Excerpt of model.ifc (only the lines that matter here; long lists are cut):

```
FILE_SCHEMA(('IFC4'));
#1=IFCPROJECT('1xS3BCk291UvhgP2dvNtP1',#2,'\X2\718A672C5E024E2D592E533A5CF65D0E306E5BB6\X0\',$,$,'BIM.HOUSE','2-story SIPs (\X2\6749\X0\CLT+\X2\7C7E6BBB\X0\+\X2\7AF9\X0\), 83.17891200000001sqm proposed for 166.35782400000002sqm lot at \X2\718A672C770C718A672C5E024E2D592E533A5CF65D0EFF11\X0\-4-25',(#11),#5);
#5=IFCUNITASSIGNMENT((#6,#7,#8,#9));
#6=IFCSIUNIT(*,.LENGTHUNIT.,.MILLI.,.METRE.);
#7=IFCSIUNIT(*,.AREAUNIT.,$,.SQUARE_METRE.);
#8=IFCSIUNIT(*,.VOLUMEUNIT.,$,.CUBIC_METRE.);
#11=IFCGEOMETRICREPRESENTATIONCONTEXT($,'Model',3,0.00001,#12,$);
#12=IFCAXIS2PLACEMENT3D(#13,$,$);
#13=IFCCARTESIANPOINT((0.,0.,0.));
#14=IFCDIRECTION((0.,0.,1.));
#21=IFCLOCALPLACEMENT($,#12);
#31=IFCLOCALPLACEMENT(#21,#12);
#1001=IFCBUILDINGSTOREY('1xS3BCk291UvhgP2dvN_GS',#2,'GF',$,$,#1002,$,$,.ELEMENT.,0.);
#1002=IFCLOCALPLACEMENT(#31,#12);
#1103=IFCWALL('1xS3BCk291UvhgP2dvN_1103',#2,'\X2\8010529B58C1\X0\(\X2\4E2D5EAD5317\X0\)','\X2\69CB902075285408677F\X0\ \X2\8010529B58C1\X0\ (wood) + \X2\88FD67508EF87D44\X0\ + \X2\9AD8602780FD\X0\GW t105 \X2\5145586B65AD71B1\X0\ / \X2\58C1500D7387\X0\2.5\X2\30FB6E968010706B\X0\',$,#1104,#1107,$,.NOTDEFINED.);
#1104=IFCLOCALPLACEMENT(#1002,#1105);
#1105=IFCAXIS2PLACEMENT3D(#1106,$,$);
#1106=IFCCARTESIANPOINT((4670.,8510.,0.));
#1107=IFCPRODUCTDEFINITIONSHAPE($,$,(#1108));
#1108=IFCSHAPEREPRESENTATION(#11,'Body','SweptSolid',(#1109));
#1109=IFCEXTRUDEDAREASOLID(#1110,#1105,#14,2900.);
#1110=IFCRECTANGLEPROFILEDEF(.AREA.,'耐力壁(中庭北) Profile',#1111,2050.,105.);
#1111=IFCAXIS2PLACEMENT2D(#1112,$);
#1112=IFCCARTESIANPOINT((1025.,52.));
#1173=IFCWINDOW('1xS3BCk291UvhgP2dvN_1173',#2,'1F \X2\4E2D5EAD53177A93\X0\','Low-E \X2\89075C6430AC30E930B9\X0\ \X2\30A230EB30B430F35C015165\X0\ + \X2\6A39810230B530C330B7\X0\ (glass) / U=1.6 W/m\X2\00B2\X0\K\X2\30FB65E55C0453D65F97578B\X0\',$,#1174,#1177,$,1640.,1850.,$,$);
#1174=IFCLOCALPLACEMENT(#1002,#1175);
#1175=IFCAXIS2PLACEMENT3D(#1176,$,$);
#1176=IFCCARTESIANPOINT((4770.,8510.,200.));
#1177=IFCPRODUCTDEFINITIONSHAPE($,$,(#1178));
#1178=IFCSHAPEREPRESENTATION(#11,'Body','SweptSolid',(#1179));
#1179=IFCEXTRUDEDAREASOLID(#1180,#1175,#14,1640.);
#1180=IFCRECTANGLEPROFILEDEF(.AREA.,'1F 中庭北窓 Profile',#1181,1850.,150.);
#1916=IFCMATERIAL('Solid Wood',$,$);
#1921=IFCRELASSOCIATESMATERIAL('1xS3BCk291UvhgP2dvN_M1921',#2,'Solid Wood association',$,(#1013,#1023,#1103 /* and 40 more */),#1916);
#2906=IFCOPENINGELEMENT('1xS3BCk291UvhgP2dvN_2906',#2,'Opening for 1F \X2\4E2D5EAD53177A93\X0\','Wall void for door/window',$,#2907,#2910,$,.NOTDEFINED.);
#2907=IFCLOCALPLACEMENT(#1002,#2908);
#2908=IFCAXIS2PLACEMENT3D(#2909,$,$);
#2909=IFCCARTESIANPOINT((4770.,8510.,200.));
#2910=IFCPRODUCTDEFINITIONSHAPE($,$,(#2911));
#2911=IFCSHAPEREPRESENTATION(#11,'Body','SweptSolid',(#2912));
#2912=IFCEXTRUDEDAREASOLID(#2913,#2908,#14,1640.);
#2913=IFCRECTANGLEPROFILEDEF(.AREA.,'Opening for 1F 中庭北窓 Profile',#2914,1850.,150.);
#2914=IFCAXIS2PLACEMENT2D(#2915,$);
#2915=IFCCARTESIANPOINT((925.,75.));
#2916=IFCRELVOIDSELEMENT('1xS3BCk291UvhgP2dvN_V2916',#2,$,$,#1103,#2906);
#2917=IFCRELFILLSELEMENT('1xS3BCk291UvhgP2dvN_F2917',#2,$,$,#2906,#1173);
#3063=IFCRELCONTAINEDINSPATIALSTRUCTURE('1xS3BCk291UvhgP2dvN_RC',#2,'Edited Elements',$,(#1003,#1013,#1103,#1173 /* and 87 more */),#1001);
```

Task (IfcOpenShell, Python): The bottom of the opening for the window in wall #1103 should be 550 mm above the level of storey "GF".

```python
import numpy as np
import ifcopenshell
import ifcopenshell.api.geometry
import ifcopenshell.geom
import ifcopenshell.util.element
import ifcopenshell.util.placement
import ifcopenshell.util.shape
import ifcopenshell.util.unit

model = ifcopenshell.open("model.ifc")
unit_scale = ifcopenshell.util.unit.calculate_unit_scale(model)

window = model.by_guid("1xS3BCk291UvhgP2dvN_1173")
opening = window.FillsVoids[0].RelatingOpeningElement
storey = ifcopenshell.util.element.get_container(window, ifc_class="IfcBuildingStorey")
level = ifcopenshell.util.placement.get_local_placement(storey.ObjectPlacement)[2, 3]

# The opening's origin need not be at the sill, so measure its lowest point.
shape = ifcopenshell.geom.create_shape(ifcopenshell.geom.settings(), opening)
bottom = ifcopenshell.util.shape.get_shape_bottom_elevation(shape, shape.geometry) / unit_scale
dz = level + 0.55 / unit_scale - bottom

shift = np.array([0.0, 0.0, dz])
# The window is not placed relative to its opening, so move both.
for product in (opening, window):
    matrix = ifcopenshell.util.placement.get_local_placement(product.ObjectPlacement)
    matrix[:3, 3] += shift
    ifcopenshell.api.geometry.edit_object_placement(model, product=product, matrix=matrix, is_si=False)

print(f"moved by {dz * unit_scale:+.3f} m")

model.write("model-out.ifc")
```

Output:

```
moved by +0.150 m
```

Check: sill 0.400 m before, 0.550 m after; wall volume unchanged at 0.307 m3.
